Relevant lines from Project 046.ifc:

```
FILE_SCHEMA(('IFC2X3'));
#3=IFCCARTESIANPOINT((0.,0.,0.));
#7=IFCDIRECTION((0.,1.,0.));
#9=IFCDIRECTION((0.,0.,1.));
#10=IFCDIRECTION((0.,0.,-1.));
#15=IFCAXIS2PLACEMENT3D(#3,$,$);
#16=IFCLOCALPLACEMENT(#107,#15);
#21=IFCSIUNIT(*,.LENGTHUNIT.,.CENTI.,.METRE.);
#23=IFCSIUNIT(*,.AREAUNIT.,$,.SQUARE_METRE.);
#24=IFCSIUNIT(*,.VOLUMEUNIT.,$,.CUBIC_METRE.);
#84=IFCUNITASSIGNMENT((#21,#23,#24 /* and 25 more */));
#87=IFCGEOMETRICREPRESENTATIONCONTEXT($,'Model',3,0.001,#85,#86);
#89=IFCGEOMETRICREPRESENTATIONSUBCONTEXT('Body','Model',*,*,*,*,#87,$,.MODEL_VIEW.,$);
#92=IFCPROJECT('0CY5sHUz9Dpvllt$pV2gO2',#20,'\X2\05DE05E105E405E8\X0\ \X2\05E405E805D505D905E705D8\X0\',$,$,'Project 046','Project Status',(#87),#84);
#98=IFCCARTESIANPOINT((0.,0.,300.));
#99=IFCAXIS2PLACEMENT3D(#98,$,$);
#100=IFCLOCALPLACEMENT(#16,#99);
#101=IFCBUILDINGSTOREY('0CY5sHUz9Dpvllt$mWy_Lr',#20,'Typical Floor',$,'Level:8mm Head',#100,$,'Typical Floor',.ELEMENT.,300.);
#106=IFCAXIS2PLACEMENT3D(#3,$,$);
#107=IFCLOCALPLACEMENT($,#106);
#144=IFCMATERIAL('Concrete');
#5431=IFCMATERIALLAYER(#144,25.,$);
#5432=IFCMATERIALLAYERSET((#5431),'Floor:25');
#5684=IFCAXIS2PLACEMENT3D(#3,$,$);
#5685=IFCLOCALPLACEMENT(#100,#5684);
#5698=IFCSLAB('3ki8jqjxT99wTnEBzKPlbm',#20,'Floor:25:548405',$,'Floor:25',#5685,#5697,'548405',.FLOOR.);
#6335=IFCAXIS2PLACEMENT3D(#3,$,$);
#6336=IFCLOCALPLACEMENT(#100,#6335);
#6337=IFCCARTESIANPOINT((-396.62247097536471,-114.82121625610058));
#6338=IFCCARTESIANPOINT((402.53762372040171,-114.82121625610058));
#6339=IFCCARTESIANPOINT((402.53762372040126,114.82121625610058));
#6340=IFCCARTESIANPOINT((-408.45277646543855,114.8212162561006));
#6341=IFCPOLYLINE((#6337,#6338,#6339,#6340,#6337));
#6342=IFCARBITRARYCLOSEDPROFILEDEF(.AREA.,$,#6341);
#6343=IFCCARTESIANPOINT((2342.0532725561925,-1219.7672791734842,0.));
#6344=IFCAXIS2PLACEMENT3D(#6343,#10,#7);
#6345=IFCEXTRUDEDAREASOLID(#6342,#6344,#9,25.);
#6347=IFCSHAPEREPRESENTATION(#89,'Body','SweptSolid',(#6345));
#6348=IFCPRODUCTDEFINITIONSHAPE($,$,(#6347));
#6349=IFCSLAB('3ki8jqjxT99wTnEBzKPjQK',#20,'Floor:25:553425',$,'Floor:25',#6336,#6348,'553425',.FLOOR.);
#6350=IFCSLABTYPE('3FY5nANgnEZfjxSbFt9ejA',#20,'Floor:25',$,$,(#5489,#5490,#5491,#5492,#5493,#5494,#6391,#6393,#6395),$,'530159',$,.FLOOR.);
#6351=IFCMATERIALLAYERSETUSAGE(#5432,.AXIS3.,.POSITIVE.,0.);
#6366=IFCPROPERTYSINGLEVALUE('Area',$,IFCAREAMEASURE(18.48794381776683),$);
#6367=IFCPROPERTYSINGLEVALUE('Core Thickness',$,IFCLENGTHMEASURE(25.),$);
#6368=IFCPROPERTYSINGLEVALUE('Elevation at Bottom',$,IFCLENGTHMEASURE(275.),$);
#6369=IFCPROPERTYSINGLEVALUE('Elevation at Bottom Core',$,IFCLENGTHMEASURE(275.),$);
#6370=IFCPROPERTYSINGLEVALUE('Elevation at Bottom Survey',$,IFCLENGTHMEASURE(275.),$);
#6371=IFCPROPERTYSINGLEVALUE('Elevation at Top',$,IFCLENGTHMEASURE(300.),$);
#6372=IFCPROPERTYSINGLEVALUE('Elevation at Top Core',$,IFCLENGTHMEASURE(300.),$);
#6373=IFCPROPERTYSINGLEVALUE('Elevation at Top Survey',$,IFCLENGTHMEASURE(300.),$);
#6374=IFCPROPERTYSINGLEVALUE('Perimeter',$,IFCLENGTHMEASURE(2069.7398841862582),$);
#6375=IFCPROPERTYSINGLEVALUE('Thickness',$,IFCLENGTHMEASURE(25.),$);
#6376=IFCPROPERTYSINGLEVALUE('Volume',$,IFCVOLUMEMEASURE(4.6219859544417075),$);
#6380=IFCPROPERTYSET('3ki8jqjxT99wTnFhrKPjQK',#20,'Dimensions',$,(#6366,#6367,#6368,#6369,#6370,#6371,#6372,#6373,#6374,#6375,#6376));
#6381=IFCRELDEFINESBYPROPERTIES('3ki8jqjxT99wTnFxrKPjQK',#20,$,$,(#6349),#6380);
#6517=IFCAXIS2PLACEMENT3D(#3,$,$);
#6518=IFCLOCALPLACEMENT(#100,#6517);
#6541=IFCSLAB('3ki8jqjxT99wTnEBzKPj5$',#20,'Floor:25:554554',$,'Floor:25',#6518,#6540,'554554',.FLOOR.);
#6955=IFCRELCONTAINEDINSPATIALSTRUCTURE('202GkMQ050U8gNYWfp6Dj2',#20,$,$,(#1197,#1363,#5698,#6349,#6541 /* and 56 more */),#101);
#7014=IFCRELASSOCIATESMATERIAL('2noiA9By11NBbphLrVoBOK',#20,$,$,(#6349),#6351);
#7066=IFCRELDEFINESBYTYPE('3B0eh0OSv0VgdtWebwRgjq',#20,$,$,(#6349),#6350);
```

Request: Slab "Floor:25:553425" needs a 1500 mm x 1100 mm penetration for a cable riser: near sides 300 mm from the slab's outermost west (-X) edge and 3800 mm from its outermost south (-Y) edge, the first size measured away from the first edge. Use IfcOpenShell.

```python
import numpy as np
import ifcopenshell
import ifcopenshell.api.feature
import ifcopenshell.api.geometry
import ifcopenshell.api.pset
import ifcopenshell.api.root
import ifcopenshell.geom
import ifcopenshell.util.element
import ifcopenshell.util.placement
import ifcopenshell.util.representation
import ifcopenshell.util.shape
import ifcopenshell.util.unit

model = ifcopenshell.open("Project 046.ifc")
unit_scale = ifcopenshell.util.unit.calculate_unit_scale(model)
area_scale = ifcopenshell.util.unit.calculate_unit_scale(model, "AREAUNIT")
volume_scale = ifcopenshell.util.unit.calculate_unit_scale(model, "VOLUMEUNIT")
settings = ifcopenshell.geom.settings()


def volume(element):
    """Net volume in cubic metres, openings subtracted."""
    shape = ifcopenshell.geom.create_shape(settings, element)
    return ifcopenshell.util.shape.get_volume(shape.geometry)


slab = model.by_guid("3ki8jqjxT99wTnEBzKPjQK")
before = volume(slab)

# Extent in the slab's own axes, in metres. The edges named are its -X and -Y sides.
slab_shape = ifcopenshell.geom.create_shape(settings, slab)
vertices = ifcopenshell.util.shape.get_vertices(slab_shape.geometry)
x_min, y_min, bottom = vertices.min(axis=0)
top = vertices[:, 2].max()

opening = ifcopenshell.api.root.create_entity(model, ifc_class="IfcOpeningElement", name="Cable riser opening")
context = ifcopenshell.util.representation.get_context(model, "Model", "Body", "MODEL_VIEW")
width, depth = 1.5, 1.1
outline = [(0.0, 0.0), (width, 0.0), (width, depth), (0.0, depth), (0.0, 0.0)]
# Overshoot both faces by 50 mm so the cut is clean.
shape = ifcopenshell.api.geometry.add_slab_representation(
    model, context=context, depth=top - bottom + 0.1, polyline=outline
)
ifcopenshell.api.geometry.assign_representation(model, product=opening, representation=shape)

matrix = ifcopenshell.util.placement.get_local_placement(slab.ObjectPlacement)
matrix[:, 3] = matrix @ np.append(np.array([x_min + 0.3, y_min + 3.8, bottom - 0.05]) / unit_scale, 1.0)
ifcopenshell.api.geometry.edit_object_placement(model, product=opening, matrix=matrix, is_si=False)
ifcopenshell.api.feature.add_feature(model, feature=opening, element=slab)

after = volume(slab)

# Update the slab's stored quantities.
pset = model.by_id(ifcopenshell.util.element.get_pset(slab, "Dimensions", should_inherit=False)["id"])
ifcopenshell.api.pset.edit_pset(model, pset=pset, properties={
    "Area": model.create_entity("IfcAreaMeasure", after / (top - bottom) / area_scale),
    "Volume": model.create_entity("IfcVolumeMeasure", after / volume_scale),
})

print(f"slab volume {before:.3f} -> {after:.3f} m3")

model.write("Project 046_updated.ifc")
```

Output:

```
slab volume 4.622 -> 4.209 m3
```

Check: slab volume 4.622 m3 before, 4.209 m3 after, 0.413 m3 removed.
